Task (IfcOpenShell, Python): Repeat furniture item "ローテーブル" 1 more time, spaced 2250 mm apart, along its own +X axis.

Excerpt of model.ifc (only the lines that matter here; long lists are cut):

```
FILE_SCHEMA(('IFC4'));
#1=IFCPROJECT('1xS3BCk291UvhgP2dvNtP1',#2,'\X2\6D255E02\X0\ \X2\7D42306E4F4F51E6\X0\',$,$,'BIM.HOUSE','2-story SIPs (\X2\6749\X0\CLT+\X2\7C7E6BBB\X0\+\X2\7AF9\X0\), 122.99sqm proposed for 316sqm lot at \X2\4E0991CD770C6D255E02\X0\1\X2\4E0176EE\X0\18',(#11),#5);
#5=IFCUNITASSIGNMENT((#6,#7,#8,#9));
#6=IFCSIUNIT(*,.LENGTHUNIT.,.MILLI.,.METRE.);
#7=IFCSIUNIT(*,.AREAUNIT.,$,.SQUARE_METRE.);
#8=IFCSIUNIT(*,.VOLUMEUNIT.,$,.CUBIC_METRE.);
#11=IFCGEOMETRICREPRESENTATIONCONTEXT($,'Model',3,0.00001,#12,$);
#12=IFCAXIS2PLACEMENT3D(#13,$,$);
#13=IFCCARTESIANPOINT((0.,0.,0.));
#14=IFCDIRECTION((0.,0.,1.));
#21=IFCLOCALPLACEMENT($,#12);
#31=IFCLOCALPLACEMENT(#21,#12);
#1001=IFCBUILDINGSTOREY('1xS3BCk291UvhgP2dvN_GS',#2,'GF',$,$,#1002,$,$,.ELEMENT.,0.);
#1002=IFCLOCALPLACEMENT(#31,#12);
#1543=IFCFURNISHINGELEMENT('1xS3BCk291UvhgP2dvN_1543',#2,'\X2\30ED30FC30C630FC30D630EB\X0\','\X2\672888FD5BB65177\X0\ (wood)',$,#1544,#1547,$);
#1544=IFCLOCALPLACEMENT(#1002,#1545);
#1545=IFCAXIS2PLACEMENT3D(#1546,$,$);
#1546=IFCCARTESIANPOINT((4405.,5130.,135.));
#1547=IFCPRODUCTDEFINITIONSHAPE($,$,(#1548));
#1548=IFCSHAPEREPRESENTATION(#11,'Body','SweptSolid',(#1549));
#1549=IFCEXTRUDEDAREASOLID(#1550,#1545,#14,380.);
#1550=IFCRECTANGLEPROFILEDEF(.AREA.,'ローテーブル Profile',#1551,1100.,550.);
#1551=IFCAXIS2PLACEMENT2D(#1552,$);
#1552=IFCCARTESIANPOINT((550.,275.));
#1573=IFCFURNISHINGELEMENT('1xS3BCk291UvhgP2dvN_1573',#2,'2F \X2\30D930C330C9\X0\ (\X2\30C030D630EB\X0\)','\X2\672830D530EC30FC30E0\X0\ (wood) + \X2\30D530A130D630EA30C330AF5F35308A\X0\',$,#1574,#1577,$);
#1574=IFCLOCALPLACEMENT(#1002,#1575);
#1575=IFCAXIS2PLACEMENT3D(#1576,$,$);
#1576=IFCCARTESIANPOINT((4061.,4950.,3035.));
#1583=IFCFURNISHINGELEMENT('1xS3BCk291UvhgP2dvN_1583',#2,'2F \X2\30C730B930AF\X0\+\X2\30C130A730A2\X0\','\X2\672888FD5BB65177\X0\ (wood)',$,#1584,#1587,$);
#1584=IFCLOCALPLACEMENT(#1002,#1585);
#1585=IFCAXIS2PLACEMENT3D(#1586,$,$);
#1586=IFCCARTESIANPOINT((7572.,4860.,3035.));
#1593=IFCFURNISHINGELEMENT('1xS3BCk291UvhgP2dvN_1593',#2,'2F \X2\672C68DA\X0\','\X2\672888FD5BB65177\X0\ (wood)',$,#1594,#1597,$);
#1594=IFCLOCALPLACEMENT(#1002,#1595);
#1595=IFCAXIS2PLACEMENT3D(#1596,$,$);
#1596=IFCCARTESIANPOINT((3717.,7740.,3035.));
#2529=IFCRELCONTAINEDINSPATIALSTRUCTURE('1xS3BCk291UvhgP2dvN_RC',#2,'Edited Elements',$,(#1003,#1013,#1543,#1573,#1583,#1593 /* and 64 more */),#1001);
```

```python
import ifcopenshell
import ifcopenshell.api.geometry
import ifcopenshell.api.root
import ifcopenshell.util.element
import ifcopenshell.util.placement
import ifcopenshell.util.unit

model = ifcopenshell.open("model.ifc")
unit_scale = ifcopenshell.util.unit.calculate_unit_scale(model)


def reuse_history(source, copy):
    """copy_class also copies each property set's owner history, people and application; keep the originals."""
    for rel in copy.IsDefinedBy:
        if rel.is_a("IfcRelDefinesByProperties") and (history := rel.RelatingPropertyDefinition.OwnerHistory):
            rel.RelatingPropertyDefinition.OwnerHistory = source.OwnerHistory
            ifcopenshell.util.element.remove_deep2(model, history)


source = model.by_guid("1xS3BCk291UvhgP2dvN_1543")
base = ifcopenshell.util.placement.get_local_placement(source.ObjectPlacement)
step = base[:3, 0] * 2.25 / unit_scale

for i in range(1, 2):
    copy = ifcopenshell.api.root.copy_class(model, product=source)
    copy.Representation = ifcopenshell.util.element.copy_deep(
        model, source.Representation, exclude=["IfcGeometricRepresentationContext", "IfcRepresentationMap"]
    )
    reuse_history(source, copy)
    matrix = base.copy()
    matrix[:3, 3] += i * step
    print("added at", matrix[:3, 3].round(3) + 0.0)
    ifcopenshell.api.geometry.edit_object_placement(model, product=copy, matrix=matrix, is_si=False)

model.write("model_edited.ifc")
```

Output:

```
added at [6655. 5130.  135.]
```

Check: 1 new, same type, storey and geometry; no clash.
